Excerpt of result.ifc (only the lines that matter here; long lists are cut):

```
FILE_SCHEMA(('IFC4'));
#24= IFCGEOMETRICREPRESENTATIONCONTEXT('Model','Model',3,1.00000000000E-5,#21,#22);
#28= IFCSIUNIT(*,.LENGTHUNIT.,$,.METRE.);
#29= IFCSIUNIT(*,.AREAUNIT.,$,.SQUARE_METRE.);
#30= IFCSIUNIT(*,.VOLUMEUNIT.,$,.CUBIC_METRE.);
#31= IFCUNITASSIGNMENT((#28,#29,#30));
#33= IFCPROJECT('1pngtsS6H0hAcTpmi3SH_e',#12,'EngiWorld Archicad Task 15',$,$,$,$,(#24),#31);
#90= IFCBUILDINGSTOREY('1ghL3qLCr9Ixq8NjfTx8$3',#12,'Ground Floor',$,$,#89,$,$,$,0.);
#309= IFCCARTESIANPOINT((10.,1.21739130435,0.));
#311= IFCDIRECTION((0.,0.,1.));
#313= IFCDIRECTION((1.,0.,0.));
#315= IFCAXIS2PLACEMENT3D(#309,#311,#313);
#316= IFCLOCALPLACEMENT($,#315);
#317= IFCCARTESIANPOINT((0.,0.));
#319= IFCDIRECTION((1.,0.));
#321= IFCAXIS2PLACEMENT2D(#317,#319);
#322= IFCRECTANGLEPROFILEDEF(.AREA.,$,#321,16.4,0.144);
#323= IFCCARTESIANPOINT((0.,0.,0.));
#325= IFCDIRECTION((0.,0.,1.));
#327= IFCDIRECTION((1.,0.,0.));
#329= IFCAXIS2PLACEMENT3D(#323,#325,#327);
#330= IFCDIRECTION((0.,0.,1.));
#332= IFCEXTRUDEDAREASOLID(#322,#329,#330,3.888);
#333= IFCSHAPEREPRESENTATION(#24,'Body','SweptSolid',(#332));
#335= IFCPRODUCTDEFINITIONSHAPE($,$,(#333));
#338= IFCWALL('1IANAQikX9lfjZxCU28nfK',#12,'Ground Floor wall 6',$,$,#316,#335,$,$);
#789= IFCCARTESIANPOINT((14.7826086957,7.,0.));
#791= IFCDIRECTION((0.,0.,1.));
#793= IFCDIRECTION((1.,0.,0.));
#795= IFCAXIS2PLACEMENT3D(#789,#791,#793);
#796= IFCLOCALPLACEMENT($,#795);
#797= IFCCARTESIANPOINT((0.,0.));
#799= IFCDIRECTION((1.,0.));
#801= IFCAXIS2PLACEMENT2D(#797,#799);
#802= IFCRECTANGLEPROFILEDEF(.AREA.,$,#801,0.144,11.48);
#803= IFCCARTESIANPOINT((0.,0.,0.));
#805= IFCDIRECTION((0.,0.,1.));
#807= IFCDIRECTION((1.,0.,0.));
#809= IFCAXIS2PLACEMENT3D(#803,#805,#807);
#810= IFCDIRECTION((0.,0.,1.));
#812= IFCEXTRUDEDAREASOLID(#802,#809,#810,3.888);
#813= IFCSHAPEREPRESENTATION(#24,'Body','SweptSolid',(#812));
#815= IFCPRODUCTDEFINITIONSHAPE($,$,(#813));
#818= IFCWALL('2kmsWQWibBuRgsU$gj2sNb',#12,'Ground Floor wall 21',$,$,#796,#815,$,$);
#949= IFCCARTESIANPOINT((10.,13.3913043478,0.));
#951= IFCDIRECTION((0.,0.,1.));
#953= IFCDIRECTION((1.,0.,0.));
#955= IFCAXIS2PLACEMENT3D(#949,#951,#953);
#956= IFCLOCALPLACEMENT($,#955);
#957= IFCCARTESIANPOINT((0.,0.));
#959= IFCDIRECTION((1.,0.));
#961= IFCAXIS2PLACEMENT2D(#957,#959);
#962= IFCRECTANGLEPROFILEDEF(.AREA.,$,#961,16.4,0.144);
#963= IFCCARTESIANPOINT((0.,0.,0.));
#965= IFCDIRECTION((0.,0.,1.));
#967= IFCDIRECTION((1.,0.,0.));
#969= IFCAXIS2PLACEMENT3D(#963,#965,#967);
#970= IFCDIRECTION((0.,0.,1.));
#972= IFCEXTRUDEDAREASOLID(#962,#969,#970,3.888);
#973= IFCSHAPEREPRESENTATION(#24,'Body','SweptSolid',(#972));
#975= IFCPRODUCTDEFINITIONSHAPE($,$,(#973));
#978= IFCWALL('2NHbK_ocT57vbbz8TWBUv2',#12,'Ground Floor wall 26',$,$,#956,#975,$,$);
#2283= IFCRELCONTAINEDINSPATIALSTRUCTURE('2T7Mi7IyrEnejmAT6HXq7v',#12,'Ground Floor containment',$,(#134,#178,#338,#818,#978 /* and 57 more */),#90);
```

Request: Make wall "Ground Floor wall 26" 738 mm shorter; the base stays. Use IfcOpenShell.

```python
import ifcopenshell
import ifcopenshell.geom
import ifcopenshell.util.shape

model = ifcopenshell.open("result.ifc")
settings = ifcopenshell.geom.settings()


def volume(element):
    """Net volume in cubic metres, openings subtracted."""
    shape = ifcopenshell.geom.create_shape(settings, element)
    return ifcopenshell.util.shape.get_volume(shape.geometry)


wall = model.by_guid("2NHbK_ocT57vbbz8TWBUv2")
before = volume(wall)

body = next(r for r in wall.Representation.Representations if r.RepresentationIdentifier == "Body")
solid = body.Items[0]
old_height = solid.Depth
solid.Depth -= 0.738
after = volume(wall)

print(f"height {old_height:g} -> {solid.Depth:g}, volume {before:.3f} -> {after:.3f} m3")

model.write("result_rev.ifc")
```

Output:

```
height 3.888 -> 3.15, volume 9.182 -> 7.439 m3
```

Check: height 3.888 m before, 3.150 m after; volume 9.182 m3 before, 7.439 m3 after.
